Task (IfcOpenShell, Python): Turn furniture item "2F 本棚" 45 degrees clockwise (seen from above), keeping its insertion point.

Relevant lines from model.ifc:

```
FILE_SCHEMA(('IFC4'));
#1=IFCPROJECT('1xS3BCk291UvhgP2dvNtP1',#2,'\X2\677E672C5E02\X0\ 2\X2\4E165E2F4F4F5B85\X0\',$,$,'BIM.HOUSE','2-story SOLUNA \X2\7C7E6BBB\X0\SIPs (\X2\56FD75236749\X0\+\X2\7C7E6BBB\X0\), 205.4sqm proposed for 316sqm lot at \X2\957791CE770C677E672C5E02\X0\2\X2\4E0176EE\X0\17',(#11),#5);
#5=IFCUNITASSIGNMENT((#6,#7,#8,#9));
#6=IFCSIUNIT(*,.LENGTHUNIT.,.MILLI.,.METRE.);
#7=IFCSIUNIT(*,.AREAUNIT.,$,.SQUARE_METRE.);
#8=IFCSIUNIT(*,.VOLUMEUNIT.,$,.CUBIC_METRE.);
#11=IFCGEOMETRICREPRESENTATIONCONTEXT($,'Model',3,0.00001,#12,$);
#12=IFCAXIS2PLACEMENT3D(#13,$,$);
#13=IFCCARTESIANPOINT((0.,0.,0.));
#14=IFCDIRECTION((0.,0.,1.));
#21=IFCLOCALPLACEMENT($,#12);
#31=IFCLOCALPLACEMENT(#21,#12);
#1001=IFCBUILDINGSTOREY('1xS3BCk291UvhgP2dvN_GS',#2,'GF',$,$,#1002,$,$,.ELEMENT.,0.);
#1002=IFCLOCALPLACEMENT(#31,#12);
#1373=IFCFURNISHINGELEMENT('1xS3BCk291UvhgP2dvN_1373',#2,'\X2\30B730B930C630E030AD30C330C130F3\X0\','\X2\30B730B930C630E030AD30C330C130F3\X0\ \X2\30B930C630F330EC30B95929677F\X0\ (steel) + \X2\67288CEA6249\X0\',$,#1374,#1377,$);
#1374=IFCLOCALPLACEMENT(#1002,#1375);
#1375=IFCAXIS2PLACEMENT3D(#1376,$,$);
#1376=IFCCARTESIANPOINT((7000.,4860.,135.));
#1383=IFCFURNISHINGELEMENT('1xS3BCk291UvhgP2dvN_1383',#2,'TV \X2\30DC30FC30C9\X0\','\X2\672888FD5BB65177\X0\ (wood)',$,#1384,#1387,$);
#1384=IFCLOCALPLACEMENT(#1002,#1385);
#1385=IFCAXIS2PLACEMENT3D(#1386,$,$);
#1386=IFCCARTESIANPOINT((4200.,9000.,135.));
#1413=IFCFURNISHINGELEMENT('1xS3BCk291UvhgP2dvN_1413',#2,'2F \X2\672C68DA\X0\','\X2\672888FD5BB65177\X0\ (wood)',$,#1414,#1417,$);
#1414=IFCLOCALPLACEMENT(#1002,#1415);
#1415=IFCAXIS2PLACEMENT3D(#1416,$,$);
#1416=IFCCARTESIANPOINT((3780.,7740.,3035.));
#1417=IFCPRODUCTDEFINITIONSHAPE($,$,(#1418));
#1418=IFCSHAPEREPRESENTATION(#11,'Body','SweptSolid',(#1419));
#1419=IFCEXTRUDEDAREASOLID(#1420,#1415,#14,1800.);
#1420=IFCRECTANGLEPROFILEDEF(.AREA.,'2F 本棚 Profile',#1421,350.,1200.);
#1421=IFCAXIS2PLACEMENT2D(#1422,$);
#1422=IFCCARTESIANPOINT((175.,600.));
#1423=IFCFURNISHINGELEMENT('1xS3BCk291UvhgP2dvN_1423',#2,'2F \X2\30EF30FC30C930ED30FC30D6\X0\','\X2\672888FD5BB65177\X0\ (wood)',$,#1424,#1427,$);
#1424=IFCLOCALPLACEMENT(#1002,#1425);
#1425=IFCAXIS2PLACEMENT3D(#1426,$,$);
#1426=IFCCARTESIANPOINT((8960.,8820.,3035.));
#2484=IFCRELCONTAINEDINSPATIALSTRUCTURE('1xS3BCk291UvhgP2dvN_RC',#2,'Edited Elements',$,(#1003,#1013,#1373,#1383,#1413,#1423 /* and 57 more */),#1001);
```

```python
import ifcopenshell
import ifcopenshell.api.geometry
import ifcopenshell.util.placement

model = ifcopenshell.open("model.ifc")

item = model.by_id(1413)
matrix = ifcopenshell.util.placement.get_local_placement(item.ObjectPlacement)
matrix = matrix @ ifcopenshell.util.placement.rotation(-45, "Z")
ifcopenshell.api.geometry.edit_object_placement(model, product=item, matrix=matrix, is_si=False)

print(ifcopenshell.util.placement.get_local_placement(item.ObjectPlacement).round(3) + 0.0)

model.write("model_edited.ifc")
```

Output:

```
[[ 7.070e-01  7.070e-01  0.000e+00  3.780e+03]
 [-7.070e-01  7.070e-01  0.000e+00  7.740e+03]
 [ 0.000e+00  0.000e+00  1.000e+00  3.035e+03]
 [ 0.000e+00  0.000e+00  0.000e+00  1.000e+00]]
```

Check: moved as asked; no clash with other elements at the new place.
